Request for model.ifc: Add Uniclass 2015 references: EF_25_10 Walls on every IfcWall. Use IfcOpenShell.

First a look at what the model holds.

```python
import ifcopenshell

model = ifcopenshell.open("model.ifc")
print(model.schema)
print("classifications:", [c.Name for c in model.by_type("IfcClassification")])
for ifc_class in ("IfcDoor", "IfcRoof", "IfcStair", "IfcWall", "IfcWindow"):
    print(ifc_class, len(model.by_type(ifc_class)))
```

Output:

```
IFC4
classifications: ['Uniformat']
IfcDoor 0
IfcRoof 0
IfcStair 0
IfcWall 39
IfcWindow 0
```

```python
import ifcopenshell
import ifcopenshell.api.classification

model = ifcopenshell.open("model.ifc")

system = ifcopenshell.api.classification.add_classification(model, classification="Uniclass 2015")

codes = {
    "IfcWall": ("EF_25_10", "Walls"),
}
for ifc_class, (code, name) in codes.items():
    products = model.by_type(ifc_class)
    ifcopenshell.api.classification.add_reference(
        model, products=products, classification=system, identification=code, name=name
    )
    print(code, len(products))

model.write("model_rev.ifc")
```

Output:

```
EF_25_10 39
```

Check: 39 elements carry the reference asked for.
